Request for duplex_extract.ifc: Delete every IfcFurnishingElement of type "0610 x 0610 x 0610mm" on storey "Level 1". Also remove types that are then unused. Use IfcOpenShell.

First a look at what the model holds.

```python
import ifcopenshell
import ifcopenshell.util.element

model = ifcopenshell.open("duplex_extract.ifc")
print(model.schema)
storey = next(s for s in model.by_type("IfcBuildingStorey") if s.Name == "Level 1")
furniture = [e for e in ifcopenshell.util.element.get_decomposition(storey) if e.is_a("IfcFurnishingElement")]
seen = {}
for e in furniture:
    element_type = ifcopenshell.util.element.get_type(e)
    name = element_type.Name if element_type not in (None, e) else None
    seen[name] = seen.get(name, 0) + 1
for name, count in sorted(seen.items(), key=str):
    print(count, "x", name)
```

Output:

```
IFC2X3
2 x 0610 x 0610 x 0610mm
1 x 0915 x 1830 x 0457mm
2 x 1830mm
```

```python
import ifcopenshell
import ifcopenshell.api.root
import ifcopenshell.util.element

model = ifcopenshell.open("duplex_extract.ifc")

storey = next(s for s in model.by_type("IfcBuildingStorey") if s.Name == "Level 1")
furniture = [e for e in ifcopenshell.util.element.get_decomposition(storey) if e.is_a("IfcFurnishingElement")]
targets = [e for e in furniture if (t := ifcopenshell.util.element.get_type(e)) not in (None, e) and t.Name == "0610 x 0610 x 0610mm"]
types = {ifcopenshell.util.element.get_type(e) for e in targets} - {None, *targets}

for e in targets:
    ifcopenshell.api.root.remove_product(model, product=e)
print(len(targets), "removed")

unused = [t for t in types if not ifcopenshell.util.element.get_types(t)]
for t in unused:
    ifcopenshell.api.root.remove_product(model, product=t)
print(len(unused), "unused types removed")

model.write("duplex_extract_rev.ifc")
```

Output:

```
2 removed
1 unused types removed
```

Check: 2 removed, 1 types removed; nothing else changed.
